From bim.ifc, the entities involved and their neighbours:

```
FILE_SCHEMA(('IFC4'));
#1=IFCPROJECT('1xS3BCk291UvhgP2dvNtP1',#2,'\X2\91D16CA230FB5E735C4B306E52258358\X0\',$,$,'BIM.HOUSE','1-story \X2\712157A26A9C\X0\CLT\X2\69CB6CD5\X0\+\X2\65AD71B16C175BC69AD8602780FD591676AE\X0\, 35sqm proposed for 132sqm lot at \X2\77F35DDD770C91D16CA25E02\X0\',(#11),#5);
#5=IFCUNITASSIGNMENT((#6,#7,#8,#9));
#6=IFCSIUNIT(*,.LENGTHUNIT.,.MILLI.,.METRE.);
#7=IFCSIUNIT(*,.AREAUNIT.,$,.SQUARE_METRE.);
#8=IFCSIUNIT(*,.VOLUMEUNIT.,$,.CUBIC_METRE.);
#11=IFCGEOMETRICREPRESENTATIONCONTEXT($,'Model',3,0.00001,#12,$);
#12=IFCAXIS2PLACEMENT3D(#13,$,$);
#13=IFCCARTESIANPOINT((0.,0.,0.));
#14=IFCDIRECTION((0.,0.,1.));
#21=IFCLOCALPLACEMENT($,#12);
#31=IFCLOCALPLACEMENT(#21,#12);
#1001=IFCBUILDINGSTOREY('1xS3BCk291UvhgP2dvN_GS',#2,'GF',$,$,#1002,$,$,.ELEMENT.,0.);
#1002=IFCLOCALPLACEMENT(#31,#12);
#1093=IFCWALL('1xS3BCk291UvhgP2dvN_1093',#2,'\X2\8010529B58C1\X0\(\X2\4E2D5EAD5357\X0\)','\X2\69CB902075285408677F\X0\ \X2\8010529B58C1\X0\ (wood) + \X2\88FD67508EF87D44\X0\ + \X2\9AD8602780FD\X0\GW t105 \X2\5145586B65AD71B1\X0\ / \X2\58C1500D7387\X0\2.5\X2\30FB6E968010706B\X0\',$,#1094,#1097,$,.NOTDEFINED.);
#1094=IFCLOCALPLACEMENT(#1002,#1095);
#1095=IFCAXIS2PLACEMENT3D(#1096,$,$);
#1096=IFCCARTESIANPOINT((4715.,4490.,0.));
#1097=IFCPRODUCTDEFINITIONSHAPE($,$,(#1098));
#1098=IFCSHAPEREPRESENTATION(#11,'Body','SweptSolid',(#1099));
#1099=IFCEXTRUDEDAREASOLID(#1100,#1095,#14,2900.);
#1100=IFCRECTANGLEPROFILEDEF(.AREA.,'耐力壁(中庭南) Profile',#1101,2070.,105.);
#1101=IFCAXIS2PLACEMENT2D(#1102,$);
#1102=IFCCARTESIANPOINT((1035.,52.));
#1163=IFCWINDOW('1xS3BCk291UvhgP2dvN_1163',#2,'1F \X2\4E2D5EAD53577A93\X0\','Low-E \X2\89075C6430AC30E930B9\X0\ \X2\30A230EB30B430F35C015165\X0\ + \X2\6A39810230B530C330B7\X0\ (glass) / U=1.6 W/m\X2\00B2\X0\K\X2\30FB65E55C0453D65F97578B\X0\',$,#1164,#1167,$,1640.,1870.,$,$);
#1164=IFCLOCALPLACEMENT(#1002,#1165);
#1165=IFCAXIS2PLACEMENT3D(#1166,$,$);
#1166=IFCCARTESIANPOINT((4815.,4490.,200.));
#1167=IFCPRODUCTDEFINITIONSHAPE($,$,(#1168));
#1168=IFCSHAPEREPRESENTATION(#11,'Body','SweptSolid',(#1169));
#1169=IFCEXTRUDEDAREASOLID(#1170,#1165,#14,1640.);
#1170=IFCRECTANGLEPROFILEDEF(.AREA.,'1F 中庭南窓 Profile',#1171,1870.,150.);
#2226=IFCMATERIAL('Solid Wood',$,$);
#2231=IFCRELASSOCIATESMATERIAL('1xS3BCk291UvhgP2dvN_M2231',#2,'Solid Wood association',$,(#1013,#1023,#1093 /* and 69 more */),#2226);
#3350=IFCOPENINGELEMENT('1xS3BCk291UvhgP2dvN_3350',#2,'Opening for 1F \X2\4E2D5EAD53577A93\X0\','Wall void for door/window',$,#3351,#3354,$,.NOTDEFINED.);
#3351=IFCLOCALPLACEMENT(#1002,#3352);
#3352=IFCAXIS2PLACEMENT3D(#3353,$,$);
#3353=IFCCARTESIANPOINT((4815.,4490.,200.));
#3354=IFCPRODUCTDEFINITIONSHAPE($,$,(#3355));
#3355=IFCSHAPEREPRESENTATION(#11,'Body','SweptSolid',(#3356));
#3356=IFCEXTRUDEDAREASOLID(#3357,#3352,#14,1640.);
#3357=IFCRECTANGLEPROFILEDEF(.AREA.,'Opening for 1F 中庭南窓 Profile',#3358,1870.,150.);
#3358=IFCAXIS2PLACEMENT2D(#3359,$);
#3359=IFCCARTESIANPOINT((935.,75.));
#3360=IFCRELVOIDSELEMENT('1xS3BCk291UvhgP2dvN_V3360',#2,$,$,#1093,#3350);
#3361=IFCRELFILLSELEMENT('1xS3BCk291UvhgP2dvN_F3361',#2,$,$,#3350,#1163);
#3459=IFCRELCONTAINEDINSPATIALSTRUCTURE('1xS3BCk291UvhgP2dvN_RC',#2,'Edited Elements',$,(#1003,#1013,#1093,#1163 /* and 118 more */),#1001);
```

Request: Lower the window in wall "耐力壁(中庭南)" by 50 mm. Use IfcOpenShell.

```python
import numpy as np
import ifcopenshell
import ifcopenshell.api.geometry
import ifcopenshell.util.placement
import ifcopenshell.util.unit

model = ifcopenshell.open("bim.ifc")
unit_scale = ifcopenshell.util.unit.calculate_unit_scale(model)

window = model.by_guid("1xS3BCk291UvhgP2dvN_1163")
opening = window.FillsVoids[0].RelatingOpeningElement
dz = -0.05 / unit_scale

shift = np.array([0.0, 0.0, dz])
# The window is not placed relative to its opening, so move both.
for product in (opening, window):
    matrix = ifcopenshell.util.placement.get_local_placement(product.ObjectPlacement)
    matrix[:3, 3] += shift
    ifcopenshell.api.geometry.edit_object_placement(model, product=product, matrix=matrix, is_si=False)

print(f"moved by {dz * unit_scale:+.3f} m")

model.write("bim_rev.ifc")
```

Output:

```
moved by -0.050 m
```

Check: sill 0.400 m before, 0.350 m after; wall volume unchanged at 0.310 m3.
